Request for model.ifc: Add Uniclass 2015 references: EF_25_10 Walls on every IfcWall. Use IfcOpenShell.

First a look at what the model holds.

```python
import ifcopenshell

model = ifcopenshell.open("model.ifc")
print(model.schema)
print("classifications:", [c.Name for c in model.by_type("IfcClassification")])
for ifc_class in ("IfcDoor", "IfcRoof", "IfcStair", "IfcWall", "IfcWindow"):
    print(ifc_class, len(model.by_type(ifc_class)))
```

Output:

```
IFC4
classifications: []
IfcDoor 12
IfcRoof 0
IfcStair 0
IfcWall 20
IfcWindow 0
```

```python
import ifcopenshell
import ifcopenshell.api.classification

model = ifcopenshell.open("model.ifc")

system = ifcopenshell.api.classification.add_classification(model, classification="Uniclass 2015")

codes = {
    "IfcWall": ("EF_25_10", "Walls"),
}
for ifc_class, (code, name) in codes.items():
    products = model.by_type(ifc_class)
    ifcopenshell.api.classification.add_reference(
        model, products=products, classification=system, identification=code, name=name
    )
    print(code, len(products))

model.write("model-out.ifc")
```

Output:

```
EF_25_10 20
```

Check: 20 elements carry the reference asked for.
